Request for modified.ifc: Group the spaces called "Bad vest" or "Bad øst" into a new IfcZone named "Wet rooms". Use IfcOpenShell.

First a look at what the model holds.

```python
import ifcopenshell

model = ifcopenshell.open("modified.ifc")
print(model.schema)
seen = {}
for space in model.by_type("IfcSpace"):
    seen[space.LongName] = seen.get(space.LongName, 0) + 1
for name, count in sorted(seen.items(), key=str):
    print(count, "x", name)
print("zones:", [z.Name for z in model.by_type("IfcZone")][:20])
```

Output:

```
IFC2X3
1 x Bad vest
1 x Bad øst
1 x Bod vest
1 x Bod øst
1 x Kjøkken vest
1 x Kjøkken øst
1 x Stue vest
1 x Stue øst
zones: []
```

```python
import ifcopenshell
import ifcopenshell.api.group
import ifcopenshell.api.root

model = ifcopenshell.open("modified.ifc")

names = {"Bad vest", "Bad øst"}
spaces = [s for s in model.by_type("IfcSpace") if s.LongName in names]

zone = ifcopenshell.api.root.create_entity(model, ifc_class="IfcZone", name="Wet rooms")
ifcopenshell.api.group.assign_group(model, products=spaces, group=zone)
print(len(spaces), "spaces in", zone.Name)

model.write("modified_v2.ifc")
```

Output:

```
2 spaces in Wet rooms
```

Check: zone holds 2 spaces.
